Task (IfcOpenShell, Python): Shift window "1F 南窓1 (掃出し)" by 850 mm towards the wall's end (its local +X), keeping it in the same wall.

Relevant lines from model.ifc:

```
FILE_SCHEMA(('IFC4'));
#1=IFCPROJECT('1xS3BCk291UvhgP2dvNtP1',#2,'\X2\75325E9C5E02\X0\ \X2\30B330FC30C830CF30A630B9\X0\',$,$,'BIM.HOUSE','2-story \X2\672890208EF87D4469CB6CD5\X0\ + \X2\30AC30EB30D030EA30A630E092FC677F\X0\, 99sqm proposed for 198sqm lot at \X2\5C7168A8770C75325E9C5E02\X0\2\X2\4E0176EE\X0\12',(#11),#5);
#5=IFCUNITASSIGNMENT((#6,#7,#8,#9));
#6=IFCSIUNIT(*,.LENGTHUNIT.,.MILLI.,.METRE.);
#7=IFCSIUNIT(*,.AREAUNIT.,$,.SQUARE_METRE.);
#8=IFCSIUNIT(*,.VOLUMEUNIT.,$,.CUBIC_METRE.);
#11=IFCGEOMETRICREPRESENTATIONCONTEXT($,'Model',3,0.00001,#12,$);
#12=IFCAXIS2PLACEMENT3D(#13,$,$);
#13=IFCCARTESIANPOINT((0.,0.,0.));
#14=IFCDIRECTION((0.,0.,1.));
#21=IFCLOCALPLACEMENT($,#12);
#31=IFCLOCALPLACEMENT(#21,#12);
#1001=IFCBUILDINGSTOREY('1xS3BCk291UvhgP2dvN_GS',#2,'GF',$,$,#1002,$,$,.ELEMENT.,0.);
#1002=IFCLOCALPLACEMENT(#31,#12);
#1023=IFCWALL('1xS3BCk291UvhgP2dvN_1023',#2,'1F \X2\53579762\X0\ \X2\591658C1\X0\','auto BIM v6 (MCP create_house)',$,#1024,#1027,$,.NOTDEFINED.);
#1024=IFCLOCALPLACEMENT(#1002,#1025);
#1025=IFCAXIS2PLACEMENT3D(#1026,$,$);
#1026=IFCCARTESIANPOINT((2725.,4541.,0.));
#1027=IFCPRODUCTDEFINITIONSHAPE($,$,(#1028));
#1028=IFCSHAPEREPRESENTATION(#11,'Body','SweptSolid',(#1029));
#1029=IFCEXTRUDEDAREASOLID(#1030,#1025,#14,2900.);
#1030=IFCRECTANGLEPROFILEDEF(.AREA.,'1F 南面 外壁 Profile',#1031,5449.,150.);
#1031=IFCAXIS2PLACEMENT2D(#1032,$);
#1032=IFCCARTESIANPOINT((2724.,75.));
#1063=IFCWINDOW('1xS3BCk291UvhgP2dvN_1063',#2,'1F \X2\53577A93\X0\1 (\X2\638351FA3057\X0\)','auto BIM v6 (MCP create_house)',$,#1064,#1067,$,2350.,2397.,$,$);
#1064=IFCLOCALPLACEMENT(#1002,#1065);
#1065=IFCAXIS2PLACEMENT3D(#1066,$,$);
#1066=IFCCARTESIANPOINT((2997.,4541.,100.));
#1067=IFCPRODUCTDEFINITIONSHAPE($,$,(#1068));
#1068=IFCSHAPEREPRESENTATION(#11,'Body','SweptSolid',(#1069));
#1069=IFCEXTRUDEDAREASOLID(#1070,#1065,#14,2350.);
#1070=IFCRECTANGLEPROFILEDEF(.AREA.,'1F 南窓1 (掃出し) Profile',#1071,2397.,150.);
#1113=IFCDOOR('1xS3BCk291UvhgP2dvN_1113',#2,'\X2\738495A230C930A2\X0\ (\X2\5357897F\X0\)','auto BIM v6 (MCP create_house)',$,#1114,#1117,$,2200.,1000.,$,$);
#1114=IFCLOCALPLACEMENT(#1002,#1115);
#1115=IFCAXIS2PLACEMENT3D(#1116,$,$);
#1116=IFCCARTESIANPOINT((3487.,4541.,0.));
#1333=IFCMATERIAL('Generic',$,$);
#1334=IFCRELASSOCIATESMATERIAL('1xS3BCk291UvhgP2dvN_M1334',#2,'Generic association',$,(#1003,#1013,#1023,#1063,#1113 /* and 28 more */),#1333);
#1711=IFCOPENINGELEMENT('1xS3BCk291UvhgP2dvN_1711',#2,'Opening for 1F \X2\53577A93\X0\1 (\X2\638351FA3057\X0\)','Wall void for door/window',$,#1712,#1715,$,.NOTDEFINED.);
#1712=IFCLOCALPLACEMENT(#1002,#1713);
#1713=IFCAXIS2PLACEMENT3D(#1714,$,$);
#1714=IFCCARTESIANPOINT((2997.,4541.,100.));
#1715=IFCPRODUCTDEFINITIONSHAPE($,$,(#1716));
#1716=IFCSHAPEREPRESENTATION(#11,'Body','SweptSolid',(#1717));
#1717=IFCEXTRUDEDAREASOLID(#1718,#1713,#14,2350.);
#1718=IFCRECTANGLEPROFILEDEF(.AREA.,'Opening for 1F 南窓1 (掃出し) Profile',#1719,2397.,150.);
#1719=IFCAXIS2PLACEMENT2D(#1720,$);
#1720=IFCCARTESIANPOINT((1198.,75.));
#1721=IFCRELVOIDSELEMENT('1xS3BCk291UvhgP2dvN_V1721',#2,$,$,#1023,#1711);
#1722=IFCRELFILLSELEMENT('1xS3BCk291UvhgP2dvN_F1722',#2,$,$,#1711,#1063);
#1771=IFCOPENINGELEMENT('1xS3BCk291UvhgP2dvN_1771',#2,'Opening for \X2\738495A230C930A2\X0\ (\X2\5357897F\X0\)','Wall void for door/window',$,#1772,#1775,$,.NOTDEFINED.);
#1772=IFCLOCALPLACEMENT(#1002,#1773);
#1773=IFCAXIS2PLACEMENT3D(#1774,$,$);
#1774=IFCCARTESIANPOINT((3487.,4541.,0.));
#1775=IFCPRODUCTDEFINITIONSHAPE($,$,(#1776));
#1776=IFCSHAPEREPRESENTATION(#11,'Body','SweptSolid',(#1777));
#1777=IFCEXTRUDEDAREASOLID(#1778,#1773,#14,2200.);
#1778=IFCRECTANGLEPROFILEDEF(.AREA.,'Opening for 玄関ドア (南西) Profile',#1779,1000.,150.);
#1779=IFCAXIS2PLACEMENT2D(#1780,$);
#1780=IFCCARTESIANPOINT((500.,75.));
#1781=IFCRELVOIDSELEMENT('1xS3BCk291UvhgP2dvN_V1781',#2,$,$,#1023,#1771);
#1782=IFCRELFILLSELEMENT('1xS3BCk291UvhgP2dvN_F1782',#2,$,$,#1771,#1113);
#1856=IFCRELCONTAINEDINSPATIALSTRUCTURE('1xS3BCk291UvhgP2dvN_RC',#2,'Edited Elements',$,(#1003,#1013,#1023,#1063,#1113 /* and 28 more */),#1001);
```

```python
import ifcopenshell
import ifcopenshell.api.geometry
import ifcopenshell.util.placement
import ifcopenshell.util.unit

model = ifcopenshell.open("model.ifc")
unit_scale = ifcopenshell.util.unit.calculate_unit_scale(model)

window = model.by_id(1063)
opening = window.FillsVoids[0].RelatingOpeningElement
wall = opening.VoidsElements[0].RelatingBuildingElement

wall_matrix = ifcopenshell.util.placement.get_local_placement(wall.ObjectPlacement)
shift = wall_matrix[:3, 0] * 0.85 / unit_scale
before = ifcopenshell.util.placement.get_local_placement(window.ObjectPlacement)[:3, 3].copy()

# The window is not placed relative to its opening, so move both.
for product in (opening, window):
    matrix = ifcopenshell.util.placement.get_local_placement(product.ObjectPlacement)
    matrix[:3, 3] += shift
    ifcopenshell.api.geometry.edit_object_placement(model, product=product, matrix=matrix, is_si=False)

after = ifcopenshell.util.placement.get_local_placement(window.ObjectPlacement)[:3, 3]
print("window moved by", (after - before).round(3) + 0.0)

model.write("model-out.ifc")
```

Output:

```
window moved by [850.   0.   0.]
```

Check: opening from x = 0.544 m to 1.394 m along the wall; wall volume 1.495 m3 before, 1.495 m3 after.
